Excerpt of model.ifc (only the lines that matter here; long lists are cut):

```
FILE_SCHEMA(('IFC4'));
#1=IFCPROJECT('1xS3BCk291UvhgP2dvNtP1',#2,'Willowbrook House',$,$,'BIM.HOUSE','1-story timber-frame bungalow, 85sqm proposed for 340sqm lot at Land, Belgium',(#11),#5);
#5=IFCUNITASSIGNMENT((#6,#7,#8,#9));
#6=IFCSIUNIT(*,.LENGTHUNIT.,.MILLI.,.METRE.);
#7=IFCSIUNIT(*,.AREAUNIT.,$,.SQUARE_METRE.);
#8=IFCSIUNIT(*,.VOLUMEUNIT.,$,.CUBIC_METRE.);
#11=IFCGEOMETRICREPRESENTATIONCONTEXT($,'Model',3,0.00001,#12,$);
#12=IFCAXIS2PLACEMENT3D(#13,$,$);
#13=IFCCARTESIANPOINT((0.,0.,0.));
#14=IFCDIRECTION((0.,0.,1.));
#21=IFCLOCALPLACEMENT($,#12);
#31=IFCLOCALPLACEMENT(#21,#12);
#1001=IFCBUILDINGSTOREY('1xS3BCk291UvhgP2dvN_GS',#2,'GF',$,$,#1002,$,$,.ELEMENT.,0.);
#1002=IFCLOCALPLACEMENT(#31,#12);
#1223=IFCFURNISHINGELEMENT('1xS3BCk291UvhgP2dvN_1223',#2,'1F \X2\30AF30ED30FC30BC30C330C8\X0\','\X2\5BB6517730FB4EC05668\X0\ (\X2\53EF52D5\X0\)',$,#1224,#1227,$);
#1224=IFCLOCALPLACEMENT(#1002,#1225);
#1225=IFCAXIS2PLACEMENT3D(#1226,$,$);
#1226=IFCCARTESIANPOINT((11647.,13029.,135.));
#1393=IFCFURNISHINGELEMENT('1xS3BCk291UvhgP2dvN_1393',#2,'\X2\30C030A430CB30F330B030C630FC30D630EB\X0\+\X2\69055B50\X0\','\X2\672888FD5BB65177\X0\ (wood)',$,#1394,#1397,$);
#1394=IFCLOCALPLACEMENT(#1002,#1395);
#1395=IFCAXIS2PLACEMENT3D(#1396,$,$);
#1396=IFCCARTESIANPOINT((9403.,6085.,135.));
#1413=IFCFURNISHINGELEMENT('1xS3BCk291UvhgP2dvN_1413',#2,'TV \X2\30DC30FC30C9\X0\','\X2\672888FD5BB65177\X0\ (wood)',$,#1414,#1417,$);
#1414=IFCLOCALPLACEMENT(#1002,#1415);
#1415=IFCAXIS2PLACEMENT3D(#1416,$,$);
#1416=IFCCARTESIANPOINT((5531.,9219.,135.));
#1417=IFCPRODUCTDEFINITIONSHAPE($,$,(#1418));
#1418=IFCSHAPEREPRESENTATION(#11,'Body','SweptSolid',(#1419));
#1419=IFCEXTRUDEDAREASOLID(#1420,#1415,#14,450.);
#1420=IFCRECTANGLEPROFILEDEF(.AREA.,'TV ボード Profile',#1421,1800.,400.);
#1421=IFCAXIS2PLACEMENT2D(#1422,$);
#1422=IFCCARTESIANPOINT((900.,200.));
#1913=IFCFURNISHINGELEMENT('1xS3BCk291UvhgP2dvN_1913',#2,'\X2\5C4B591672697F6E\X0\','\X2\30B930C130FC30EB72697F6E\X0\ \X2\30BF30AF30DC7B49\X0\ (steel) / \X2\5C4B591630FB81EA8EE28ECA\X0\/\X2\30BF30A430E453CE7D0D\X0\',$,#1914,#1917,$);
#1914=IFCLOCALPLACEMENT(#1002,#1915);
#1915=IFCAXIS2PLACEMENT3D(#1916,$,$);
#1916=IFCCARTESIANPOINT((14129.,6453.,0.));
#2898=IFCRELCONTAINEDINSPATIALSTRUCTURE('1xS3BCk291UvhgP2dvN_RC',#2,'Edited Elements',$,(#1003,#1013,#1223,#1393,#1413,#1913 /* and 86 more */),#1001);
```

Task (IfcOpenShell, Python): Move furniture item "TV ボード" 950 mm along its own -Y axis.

```python
import ifcopenshell
import ifcopenshell.api.geometry
import ifcopenshell.util.placement
import ifcopenshell.util.unit

model = ifcopenshell.open("model.ifc")
unit_scale = ifcopenshell.util.unit.calculate_unit_scale(model)

item = model.by_guid("1xS3BCk291UvhgP2dvN_1413")
matrix = ifcopenshell.util.placement.get_local_placement(item.ObjectPlacement)
matrix[:3, 3] -= matrix[:3, 1] * 0.95 / unit_scale
ifcopenshell.api.geometry.edit_object_placement(model, product=item, matrix=matrix, is_si=False)

print(ifcopenshell.util.placement.get_local_placement(item.ObjectPlacement).round(3) + 0.0)

model.write("model_v2.ifc")
```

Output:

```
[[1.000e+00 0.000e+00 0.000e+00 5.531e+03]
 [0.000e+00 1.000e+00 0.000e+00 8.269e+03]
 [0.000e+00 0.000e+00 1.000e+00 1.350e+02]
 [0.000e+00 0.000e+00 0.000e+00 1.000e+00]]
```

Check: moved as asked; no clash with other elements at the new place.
